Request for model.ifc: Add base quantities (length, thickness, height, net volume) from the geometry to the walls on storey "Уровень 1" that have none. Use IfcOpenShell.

First a look at what the model holds.

```python
import ifcopenshell
import ifcopenshell.util.element
import ifcopenshell.util.unit

model = ifcopenshell.open("model.ifc")
print(model.schema)
for unit_type in ("LENGTHUNIT", "AREAUNIT", "VOLUMEUNIT"):
    print(unit_type, ifcopenshell.util.unit.calculate_unit_scale(model, unit_type))
storey = next(s for s in model.by_type("IfcBuildingStorey") if s.Name == "Уровень 1")
walls = [e for e in ifcopenshell.util.element.get_decomposition(storey) if e.is_a("IfcWall")]
for e in sorted(walls, key=lambda e: e.id()):
    print(e.id(), e.is_a(), e.Name, list(ifcopenshell.util.element.get_psets(e, qtos_only=True)), sep=" | ")
```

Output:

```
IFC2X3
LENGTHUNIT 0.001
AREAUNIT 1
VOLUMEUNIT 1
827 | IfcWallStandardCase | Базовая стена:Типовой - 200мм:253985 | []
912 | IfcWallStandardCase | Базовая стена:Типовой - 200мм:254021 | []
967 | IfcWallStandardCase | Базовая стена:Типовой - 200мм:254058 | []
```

```python
import ifcopenshell
import ifcopenshell.api.pset
import ifcopenshell.geom
import ifcopenshell.util.element
import ifcopenshell.util.shape
import ifcopenshell.util.unit

model = ifcopenshell.open("model.ifc")
unit_scale = ifcopenshell.util.unit.calculate_unit_scale(model)
volume_scale = ifcopenshell.util.unit.calculate_unit_scale(model, "VOLUMEUNIT")
settings = ifcopenshell.geom.settings()

storey = next(s for s in model.by_type("IfcBuildingStorey") if s.Name == "Уровень 1")
walls = [e for e in ifcopenshell.util.element.get_decomposition(storey) if e.is_a("IfcWall")]

for e in sorted(walls, key=lambda e: e.id()):
    if ifcopenshell.util.element.get_psets(e, qtos_only=True, should_inherit=False):
        continue
    # Geometry comes back in metres, in the element's own axes.
    shape = ifcopenshell.geom.create_shape(settings, e)
    values = {
        "Length": ifcopenshell.util.shape.get_x(shape.geometry) / unit_scale,
        "Width": ifcopenshell.util.shape.get_y(shape.geometry) / unit_scale,
        "Height": ifcopenshell.util.shape.get_z(shape.geometry) / unit_scale,
        "NetVolume": ifcopenshell.util.shape.get_volume(shape.geometry) / volume_scale,
    }
    qto = ifcopenshell.api.pset.add_qto(model, product=e, name="BaseQuantities")
    ifcopenshell.api.pset.edit_qto(model, qto=qto, properties=values)
    print(e.id(), {k: round(v, 3) for k, v in values.items()})

model.write("model-out.ifc")
```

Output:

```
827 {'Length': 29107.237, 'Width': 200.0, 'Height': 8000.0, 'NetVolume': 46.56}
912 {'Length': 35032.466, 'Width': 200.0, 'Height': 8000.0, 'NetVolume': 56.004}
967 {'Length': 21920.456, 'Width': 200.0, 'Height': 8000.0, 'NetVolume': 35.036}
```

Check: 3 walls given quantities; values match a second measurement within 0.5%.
